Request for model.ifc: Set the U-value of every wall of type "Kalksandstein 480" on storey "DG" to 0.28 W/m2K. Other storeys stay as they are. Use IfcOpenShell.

First a look at what the model holds.

```python
import ifcopenshell
import ifcopenshell.util.element

model = ifcopenshell.open("model.ifc")
print(model.schema)
storey = next(s for s in model.by_type("IfcBuildingStorey") if s.Name == "DG")
walls = [e for e in ifcopenshell.util.element.get_decomposition(storey) if e.is_a("IfcWall")]
seen = {}
for e in walls:
    element_type = ifcopenshell.util.element.get_type(e)
    key = (element_type.Name if element_type != e and element_type else None, ifcopenshell.util.element.get_pset(e, "Pset_WallCommon", "ThermalTransmittance"))
    seen[key] = seen.get(key, 0) + 1
for (name, value), count in sorted(seen.items(), key=str):
    print(count, "x", name, "|", value)
```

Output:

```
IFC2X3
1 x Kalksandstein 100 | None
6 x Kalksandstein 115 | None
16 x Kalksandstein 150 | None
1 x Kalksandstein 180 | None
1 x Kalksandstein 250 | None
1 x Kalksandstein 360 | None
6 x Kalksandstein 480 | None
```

```python
import ifcopenshell
import ifcopenshell.api.pset
import ifcopenshell.util.element

model = ifcopenshell.open("model.ifc")

storey = next(s for s in model.by_type("IfcBuildingStorey") if s.Name == "DG")
walls = [e for e in ifcopenshell.util.element.get_decomposition(storey) if e.is_a("IfcWall")]

count = 0
for e in walls:
    element_type = ifcopenshell.util.element.get_type(e)
    if element_type in (None, e) or element_type.Name != "Kalksandstein 480":
        continue
    # add_pset returns the element's existing set when there is one.
    pset = ifcopenshell.api.pset.add_pset(model, product=e, name="Pset_WallCommon")
    ifcopenshell.api.pset.edit_pset(model, pset=pset, properties={"ThermalTransmittance": 0.28})
    count += 1

print(count, "walls updated")

model.write("model_v2.ifc")
```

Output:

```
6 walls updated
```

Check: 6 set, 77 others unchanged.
